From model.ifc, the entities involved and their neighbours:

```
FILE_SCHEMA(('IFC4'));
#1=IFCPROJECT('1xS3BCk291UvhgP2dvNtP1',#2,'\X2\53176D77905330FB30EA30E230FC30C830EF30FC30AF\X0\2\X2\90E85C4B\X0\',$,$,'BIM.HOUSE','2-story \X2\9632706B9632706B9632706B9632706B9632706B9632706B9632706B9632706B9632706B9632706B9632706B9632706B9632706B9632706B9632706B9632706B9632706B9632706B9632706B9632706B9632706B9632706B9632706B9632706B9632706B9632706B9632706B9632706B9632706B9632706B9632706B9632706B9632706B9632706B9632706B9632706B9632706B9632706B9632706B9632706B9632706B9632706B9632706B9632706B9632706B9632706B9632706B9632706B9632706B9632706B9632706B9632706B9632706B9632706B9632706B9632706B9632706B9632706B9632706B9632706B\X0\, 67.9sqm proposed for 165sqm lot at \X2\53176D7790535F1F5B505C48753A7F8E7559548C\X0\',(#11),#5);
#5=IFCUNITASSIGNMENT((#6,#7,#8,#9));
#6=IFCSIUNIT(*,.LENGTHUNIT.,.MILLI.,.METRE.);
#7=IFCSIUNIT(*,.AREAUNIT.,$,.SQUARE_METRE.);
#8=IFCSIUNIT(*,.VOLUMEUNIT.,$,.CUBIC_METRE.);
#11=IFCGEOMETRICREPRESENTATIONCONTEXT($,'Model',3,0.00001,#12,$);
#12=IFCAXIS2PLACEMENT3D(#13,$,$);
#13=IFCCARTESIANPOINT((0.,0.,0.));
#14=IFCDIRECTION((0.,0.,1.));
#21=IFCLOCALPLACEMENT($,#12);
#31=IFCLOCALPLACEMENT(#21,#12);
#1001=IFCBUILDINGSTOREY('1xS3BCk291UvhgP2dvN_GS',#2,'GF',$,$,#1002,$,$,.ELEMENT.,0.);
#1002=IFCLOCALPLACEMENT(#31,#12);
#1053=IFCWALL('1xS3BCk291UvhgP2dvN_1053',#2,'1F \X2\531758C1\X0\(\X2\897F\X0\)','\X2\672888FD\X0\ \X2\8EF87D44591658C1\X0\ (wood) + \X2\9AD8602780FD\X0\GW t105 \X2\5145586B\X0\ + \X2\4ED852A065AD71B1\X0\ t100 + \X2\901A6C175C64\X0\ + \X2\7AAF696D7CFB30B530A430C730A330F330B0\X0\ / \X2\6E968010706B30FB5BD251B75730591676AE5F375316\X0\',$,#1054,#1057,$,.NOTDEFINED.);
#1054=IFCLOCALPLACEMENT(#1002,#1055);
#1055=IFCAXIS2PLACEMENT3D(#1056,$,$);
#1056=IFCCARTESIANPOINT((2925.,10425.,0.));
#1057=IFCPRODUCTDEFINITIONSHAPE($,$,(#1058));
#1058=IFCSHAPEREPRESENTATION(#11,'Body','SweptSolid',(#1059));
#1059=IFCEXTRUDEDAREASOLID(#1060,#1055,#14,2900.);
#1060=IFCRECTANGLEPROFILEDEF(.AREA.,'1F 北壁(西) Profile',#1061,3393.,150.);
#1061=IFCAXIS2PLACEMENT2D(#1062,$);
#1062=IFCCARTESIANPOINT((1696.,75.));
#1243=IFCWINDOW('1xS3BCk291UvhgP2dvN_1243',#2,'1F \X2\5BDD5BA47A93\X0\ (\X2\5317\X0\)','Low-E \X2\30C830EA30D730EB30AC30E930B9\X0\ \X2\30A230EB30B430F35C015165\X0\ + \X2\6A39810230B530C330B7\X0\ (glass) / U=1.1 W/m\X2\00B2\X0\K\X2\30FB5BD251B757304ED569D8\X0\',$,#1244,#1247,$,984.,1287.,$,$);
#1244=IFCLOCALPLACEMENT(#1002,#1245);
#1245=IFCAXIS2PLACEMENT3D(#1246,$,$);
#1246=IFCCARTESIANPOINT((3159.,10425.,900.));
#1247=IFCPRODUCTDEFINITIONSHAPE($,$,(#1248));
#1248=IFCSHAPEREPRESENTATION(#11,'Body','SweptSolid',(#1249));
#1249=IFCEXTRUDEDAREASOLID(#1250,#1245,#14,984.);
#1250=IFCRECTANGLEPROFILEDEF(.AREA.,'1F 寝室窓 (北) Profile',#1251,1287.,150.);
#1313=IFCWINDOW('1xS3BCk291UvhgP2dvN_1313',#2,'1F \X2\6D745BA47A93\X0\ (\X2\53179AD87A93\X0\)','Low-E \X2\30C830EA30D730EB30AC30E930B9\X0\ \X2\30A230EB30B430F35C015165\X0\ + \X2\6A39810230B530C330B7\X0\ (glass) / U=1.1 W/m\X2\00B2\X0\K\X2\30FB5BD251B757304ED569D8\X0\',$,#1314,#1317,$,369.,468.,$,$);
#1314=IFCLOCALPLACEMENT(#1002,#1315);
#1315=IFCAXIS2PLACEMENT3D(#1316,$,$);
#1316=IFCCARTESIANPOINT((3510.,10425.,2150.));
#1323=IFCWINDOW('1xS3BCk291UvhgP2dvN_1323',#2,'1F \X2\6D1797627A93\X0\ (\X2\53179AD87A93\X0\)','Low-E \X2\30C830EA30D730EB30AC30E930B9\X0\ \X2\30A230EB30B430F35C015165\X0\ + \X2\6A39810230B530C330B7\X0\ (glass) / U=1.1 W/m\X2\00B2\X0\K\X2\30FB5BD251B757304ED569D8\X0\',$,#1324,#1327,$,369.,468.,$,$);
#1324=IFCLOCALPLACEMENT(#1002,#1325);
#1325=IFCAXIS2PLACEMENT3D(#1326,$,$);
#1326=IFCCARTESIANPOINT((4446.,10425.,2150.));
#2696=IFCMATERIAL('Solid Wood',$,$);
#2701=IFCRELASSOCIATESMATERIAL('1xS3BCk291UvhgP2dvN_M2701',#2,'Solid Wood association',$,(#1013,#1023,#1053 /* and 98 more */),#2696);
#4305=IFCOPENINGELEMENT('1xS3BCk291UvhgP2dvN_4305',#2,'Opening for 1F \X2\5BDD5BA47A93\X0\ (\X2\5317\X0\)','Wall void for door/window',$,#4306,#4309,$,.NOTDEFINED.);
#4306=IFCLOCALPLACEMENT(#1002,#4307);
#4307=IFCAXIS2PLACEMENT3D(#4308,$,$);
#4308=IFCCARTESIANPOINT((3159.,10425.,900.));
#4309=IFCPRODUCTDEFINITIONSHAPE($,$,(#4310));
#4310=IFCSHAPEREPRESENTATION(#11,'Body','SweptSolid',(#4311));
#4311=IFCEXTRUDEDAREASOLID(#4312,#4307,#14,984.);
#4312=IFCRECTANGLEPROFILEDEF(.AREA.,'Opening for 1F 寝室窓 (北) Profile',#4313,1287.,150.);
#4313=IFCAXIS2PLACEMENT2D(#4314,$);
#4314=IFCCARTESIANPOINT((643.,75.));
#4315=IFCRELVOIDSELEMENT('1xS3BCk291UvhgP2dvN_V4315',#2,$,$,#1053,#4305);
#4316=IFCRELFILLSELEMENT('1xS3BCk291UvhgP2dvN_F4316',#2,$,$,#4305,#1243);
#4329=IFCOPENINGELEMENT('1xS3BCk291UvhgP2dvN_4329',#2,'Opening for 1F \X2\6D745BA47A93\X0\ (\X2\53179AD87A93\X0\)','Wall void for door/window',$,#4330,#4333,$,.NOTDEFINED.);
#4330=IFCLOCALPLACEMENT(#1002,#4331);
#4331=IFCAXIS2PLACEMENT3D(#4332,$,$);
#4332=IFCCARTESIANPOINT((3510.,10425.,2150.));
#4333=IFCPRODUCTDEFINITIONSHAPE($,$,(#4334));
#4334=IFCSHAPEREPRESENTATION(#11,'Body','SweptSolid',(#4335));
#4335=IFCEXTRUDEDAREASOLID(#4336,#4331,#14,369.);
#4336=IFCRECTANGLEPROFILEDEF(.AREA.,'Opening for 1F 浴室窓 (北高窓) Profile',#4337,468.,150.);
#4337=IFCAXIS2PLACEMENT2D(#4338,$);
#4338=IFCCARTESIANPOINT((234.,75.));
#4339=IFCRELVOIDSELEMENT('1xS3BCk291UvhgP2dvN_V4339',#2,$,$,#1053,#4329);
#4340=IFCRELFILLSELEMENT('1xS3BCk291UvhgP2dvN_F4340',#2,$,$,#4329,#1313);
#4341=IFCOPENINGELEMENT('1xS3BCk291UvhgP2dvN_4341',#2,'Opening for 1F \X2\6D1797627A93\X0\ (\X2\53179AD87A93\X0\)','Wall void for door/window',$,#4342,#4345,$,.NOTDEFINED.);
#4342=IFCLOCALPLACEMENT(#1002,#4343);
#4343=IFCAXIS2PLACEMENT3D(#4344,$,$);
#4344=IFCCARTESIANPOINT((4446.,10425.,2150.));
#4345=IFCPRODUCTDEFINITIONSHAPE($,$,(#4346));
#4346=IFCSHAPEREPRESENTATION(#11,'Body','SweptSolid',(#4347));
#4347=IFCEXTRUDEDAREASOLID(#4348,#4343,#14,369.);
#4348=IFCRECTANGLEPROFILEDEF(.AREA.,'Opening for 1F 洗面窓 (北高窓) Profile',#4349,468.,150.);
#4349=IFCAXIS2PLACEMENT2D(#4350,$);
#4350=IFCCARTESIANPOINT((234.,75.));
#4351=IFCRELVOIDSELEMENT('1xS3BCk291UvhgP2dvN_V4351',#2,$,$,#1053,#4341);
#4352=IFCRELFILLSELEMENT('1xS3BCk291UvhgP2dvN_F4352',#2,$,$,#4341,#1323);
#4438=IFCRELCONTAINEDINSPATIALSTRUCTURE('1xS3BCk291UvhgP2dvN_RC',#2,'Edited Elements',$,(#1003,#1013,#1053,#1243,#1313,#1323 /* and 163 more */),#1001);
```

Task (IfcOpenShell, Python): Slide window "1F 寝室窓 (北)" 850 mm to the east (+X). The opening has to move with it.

```python
import ifcopenshell
import ifcopenshell.api.geometry
import ifcopenshell.util.placement

model = ifcopenshell.open("model.ifc")

window = model.by_guid("1xS3BCk291UvhgP2dvN_1243")
opening = window.FillsVoids[0].RelatingOpeningElement
wall = opening.VoidsElements[0].RelatingBuildingElement

wall_matrix = ifcopenshell.util.placement.get_local_placement(wall.ObjectPlacement)
shift = wall_matrix[:3, 0] * 850.0
before = ifcopenshell.util.placement.get_local_placement(window.ObjectPlacement)[:3, 3].copy()

# The window is not placed relative to its opening, so move both.
for product in (opening, window):
    matrix = ifcopenshell.util.placement.get_local_placement(product.ObjectPlacement)
    matrix[:3, 3] += shift
    ifcopenshell.api.geometry.edit_object_placement(model, product=product, matrix=matrix, is_si=False)

after = ifcopenshell.util.placement.get_local_placement(window.ObjectPlacement)[:3, 3]
print("window moved by", (after - before).round(3) + 0.0)

model.write("model-out.ifc")
```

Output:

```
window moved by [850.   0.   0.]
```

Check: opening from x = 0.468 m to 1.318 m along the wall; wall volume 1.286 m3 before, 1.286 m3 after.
